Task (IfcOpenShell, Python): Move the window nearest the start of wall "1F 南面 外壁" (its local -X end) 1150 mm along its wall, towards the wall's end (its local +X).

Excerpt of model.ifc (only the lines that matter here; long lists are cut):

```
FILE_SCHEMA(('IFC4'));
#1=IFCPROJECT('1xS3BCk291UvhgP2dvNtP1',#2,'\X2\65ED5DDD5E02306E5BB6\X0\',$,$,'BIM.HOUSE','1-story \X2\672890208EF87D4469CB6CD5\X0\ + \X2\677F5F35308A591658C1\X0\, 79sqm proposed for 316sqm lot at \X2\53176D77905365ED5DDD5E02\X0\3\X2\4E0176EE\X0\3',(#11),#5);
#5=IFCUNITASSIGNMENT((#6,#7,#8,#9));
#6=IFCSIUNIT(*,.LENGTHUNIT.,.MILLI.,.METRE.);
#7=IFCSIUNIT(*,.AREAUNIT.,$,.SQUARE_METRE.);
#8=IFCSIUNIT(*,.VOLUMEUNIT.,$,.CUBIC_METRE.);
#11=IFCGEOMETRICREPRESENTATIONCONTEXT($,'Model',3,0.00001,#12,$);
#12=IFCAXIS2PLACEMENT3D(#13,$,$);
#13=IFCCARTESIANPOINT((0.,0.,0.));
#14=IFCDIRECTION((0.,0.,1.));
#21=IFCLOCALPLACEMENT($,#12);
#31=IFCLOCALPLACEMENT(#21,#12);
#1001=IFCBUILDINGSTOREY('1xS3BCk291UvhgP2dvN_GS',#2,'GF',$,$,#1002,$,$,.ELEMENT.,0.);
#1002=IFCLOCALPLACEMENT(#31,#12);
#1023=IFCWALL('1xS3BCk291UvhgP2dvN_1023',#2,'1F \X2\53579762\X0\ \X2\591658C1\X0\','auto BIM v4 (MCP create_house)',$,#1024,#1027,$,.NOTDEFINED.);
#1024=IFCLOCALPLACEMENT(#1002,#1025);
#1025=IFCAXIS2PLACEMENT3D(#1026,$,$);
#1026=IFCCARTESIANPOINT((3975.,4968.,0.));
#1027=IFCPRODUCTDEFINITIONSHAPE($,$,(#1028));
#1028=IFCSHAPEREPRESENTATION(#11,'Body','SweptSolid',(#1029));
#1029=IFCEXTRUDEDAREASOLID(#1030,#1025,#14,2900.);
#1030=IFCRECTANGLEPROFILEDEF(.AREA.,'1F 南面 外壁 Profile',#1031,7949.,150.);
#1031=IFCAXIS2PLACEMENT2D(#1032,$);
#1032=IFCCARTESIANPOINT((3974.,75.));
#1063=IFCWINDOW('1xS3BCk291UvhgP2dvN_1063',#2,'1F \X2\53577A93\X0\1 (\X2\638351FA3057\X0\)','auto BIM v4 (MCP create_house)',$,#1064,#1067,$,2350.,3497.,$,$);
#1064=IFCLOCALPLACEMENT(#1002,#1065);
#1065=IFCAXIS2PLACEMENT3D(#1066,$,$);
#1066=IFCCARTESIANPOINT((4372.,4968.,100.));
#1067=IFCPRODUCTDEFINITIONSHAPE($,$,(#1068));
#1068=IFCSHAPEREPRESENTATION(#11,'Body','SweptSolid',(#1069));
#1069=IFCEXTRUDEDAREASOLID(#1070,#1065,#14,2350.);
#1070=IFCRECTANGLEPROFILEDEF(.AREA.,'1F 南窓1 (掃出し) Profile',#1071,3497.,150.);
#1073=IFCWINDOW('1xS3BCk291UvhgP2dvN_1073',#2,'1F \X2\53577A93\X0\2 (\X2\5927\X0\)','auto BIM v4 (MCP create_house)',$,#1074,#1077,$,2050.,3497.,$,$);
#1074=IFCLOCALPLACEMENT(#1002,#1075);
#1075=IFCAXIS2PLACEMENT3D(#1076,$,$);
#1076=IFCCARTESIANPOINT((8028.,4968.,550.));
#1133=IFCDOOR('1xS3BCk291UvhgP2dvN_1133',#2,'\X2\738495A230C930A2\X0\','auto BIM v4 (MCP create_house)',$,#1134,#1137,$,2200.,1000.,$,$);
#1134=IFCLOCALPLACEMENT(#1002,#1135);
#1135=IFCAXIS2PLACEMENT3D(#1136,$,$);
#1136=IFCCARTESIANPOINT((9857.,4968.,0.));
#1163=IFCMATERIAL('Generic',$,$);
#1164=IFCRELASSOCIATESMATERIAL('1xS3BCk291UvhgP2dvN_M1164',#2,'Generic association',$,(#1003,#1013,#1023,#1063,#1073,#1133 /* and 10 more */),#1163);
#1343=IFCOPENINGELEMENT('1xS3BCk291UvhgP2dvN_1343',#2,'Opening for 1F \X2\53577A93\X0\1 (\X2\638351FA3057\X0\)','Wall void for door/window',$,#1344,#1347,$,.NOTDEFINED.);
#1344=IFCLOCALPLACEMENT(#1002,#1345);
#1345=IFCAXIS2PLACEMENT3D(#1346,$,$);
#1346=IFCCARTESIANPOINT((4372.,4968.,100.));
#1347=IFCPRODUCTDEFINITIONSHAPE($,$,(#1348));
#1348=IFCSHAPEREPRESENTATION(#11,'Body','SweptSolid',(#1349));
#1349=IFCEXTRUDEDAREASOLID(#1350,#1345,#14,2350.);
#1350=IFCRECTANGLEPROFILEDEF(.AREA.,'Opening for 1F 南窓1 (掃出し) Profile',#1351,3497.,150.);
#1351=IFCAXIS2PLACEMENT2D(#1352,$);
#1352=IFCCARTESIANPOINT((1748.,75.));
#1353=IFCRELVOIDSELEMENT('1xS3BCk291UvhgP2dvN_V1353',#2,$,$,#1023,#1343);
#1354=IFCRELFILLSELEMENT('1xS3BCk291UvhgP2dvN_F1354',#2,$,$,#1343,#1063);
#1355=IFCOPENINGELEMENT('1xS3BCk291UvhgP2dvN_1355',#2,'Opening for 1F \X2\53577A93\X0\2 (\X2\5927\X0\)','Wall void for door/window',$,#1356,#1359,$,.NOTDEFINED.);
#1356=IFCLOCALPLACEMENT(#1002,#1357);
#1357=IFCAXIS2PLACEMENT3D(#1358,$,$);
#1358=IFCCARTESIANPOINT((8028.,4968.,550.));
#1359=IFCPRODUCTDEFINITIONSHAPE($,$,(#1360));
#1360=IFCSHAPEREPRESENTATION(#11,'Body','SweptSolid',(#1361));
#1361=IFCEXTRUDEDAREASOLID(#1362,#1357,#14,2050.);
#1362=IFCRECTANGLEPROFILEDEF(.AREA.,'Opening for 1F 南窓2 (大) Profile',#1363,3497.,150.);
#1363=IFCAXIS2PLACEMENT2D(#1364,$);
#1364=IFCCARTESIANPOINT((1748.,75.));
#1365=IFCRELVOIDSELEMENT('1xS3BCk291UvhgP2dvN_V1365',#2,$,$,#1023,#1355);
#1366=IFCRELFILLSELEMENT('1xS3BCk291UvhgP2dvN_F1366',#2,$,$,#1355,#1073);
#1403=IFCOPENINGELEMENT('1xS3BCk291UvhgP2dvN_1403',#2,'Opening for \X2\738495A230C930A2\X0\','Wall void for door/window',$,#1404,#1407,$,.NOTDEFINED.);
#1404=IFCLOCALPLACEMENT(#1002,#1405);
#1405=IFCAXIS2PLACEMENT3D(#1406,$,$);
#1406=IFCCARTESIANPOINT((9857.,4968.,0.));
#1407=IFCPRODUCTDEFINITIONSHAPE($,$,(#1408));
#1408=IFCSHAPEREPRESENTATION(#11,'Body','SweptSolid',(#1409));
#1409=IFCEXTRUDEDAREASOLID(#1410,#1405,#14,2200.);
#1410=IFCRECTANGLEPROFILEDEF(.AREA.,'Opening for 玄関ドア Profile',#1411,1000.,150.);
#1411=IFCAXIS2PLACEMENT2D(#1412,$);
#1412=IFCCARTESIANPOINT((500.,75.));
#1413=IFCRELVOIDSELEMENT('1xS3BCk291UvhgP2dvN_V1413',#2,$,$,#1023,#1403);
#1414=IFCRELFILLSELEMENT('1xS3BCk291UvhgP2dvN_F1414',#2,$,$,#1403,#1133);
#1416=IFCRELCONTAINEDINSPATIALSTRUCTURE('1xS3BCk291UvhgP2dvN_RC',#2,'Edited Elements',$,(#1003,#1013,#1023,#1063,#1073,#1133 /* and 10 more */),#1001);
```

```python
import ifcopenshell
import ifcopenshell.api.geometry
import ifcopenshell.util.placement

model = ifcopenshell.open("model.ifc")

window = model.by_guid("1xS3BCk291UvhgP2dvN_1063")
opening = window.FillsVoids[0].RelatingOpeningElement
wall = opening.VoidsElements[0].RelatingBuildingElement

wall_matrix = ifcopenshell.util.placement.get_local_placement(wall.ObjectPlacement)
shift = wall_matrix[:3, 0] * 1150.0
before = ifcopenshell.util.placement.get_local_placement(window.ObjectPlacement)[:3, 3].copy()

# The window is not placed relative to its opening, so move both.
for product in (opening, window):
    matrix = ifcopenshell.util.placement.get_local_placement(product.ObjectPlacement)
    matrix[:3, 3] += shift
    ifcopenshell.api.geometry.edit_object_placement(model, product=product, matrix=matrix, is_si=False)

after = ifcopenshell.util.placement.get_local_placement(window.ObjectPlacement)[:3, 3]
print("window moved by", (after - before).round(3) + 0.0)

model.write("model_edited.ifc")
```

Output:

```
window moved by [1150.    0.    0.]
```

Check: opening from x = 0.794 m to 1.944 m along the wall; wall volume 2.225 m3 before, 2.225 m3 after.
